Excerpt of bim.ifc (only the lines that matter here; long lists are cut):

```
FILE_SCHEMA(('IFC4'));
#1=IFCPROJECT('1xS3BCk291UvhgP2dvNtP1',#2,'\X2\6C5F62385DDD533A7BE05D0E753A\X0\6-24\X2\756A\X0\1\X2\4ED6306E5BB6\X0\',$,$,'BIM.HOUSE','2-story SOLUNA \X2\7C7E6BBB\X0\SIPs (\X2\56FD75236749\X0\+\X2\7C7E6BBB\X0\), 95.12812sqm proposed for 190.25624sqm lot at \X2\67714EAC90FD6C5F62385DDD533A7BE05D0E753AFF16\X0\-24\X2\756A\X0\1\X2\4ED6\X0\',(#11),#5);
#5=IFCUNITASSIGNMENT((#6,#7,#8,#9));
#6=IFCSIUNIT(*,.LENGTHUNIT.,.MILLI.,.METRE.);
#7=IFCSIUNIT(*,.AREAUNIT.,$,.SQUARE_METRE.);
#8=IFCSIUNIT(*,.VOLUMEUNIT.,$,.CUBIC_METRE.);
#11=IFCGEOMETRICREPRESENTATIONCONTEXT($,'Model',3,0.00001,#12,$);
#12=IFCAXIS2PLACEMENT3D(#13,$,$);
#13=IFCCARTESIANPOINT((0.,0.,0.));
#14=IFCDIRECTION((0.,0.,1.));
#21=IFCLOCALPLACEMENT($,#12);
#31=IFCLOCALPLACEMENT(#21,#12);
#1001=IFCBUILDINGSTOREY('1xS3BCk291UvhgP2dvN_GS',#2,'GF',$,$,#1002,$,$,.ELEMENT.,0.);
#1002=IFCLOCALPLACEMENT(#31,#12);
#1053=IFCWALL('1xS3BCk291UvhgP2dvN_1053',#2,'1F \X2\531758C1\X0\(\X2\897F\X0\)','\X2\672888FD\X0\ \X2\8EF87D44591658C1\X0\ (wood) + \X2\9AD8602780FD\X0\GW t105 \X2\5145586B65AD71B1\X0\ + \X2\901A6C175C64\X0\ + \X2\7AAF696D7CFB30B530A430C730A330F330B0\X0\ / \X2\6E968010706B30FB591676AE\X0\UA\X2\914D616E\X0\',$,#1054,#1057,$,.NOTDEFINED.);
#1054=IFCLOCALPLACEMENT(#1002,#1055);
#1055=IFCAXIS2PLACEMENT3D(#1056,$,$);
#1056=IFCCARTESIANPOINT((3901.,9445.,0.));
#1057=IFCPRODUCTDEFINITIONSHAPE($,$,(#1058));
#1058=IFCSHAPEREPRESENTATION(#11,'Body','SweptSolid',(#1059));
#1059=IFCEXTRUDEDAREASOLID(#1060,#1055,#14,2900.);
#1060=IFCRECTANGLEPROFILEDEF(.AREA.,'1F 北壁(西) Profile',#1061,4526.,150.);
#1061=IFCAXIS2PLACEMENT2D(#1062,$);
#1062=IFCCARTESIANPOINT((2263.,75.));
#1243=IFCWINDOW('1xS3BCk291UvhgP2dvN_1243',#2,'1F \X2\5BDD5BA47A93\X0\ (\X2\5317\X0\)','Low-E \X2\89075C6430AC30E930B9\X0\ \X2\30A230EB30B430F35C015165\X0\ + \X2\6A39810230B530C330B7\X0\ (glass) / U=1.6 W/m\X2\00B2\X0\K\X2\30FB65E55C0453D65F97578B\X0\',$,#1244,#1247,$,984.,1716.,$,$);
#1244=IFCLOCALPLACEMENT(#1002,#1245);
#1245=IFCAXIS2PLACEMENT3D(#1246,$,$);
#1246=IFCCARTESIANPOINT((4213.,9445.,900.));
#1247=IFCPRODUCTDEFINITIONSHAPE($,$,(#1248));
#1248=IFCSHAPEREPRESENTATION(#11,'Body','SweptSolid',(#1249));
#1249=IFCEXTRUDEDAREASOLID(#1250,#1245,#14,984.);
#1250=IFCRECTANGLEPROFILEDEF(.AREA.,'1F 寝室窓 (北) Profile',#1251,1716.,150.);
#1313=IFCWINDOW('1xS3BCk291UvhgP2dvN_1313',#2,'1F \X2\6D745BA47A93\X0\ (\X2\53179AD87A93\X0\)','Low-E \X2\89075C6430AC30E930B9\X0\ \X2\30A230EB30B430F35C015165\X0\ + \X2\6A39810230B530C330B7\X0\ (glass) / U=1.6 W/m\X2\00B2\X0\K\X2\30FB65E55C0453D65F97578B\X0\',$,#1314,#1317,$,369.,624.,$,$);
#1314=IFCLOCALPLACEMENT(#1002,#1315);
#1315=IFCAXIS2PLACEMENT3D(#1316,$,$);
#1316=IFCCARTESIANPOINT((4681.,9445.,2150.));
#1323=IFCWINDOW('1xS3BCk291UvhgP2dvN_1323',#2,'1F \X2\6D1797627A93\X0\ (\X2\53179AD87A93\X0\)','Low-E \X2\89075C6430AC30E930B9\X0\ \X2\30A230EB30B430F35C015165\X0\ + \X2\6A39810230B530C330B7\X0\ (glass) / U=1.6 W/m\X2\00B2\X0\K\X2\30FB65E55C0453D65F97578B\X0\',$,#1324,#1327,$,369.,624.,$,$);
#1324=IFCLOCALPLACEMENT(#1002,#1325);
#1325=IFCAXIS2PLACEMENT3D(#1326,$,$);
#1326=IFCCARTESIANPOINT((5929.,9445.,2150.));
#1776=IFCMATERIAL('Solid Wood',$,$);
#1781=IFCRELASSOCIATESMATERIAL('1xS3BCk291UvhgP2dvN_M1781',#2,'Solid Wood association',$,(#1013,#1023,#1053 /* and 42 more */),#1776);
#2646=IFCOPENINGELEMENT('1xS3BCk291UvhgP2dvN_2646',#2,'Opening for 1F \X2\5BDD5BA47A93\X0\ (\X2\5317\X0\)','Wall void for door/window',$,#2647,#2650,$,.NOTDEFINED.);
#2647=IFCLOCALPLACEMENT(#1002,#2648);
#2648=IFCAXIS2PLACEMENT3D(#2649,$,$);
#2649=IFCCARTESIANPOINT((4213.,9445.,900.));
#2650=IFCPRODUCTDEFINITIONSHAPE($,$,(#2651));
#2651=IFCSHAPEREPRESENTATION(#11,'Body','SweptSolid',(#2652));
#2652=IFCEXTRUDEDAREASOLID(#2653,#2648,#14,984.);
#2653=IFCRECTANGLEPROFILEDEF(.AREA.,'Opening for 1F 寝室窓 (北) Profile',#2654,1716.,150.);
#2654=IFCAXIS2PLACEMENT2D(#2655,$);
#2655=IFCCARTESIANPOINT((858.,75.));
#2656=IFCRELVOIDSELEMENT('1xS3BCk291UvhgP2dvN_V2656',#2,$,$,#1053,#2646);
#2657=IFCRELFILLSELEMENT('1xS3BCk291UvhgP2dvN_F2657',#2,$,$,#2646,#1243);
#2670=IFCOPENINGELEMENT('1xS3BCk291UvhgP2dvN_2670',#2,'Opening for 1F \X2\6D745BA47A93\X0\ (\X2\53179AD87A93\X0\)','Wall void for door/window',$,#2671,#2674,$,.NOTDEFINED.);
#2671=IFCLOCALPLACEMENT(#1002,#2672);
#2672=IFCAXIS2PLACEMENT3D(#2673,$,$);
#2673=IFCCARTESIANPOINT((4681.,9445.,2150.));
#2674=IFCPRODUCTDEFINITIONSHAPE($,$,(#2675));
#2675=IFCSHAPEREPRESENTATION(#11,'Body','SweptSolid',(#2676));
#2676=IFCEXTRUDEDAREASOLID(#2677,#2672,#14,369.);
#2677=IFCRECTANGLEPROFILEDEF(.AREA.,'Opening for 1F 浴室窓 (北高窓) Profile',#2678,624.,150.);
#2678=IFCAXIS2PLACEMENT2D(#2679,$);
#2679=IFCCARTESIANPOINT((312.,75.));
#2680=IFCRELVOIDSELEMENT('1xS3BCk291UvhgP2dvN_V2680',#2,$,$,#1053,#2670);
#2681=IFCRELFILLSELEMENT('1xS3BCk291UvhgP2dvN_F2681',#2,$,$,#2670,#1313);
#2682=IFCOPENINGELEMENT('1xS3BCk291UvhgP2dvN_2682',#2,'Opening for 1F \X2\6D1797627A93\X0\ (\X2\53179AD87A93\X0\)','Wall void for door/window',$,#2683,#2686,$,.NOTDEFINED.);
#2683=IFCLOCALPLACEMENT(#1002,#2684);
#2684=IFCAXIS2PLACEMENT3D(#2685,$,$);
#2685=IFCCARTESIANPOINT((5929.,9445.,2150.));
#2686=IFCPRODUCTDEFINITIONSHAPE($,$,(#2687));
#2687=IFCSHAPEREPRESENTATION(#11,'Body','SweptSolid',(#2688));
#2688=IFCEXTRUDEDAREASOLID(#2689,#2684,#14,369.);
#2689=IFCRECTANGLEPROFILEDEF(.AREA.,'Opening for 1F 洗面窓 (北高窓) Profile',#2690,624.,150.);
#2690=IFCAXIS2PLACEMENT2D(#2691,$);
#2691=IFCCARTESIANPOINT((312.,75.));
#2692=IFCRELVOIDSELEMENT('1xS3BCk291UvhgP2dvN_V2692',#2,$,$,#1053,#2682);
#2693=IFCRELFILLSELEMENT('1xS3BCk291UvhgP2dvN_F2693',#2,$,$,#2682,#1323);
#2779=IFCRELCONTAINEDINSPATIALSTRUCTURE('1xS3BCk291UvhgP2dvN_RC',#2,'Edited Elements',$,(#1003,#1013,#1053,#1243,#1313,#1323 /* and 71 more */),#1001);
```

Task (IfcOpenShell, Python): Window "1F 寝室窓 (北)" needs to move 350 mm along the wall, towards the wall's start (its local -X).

```python
import ifcopenshell
import ifcopenshell.api.geometry
import ifcopenshell.util.placement
import ifcopenshell.util.unit

model = ifcopenshell.open("bim.ifc")
unit_scale = ifcopenshell.util.unit.calculate_unit_scale(model)

window = model.by_guid("1xS3BCk291UvhgP2dvN_1243")
opening = window.FillsVoids[0].RelatingOpeningElement
wall = opening.VoidsElements[0].RelatingBuildingElement

wall_matrix = ifcopenshell.util.placement.get_local_placement(wall.ObjectPlacement)
shift = wall_matrix[:3, 0] * -0.35 / unit_scale
before = ifcopenshell.util.placement.get_local_placement(window.ObjectPlacement)[:3, 3].copy()

# The window is not placed relative to its opening, so move both.
for product in (opening, window):
    matrix = ifcopenshell.util.placement.get_local_placement(product.ObjectPlacement)
    matrix[:3, 3] += shift
    ifcopenshell.api.geometry.edit_object_placement(model, product=product, matrix=matrix, is_si=False)

after = ifcopenshell.util.placement.get_local_placement(window.ObjectPlacement)[:3, 3]
print("window moved by", (after - before).round(3) + 0.0)

model.write("bim_rev.ifc")
```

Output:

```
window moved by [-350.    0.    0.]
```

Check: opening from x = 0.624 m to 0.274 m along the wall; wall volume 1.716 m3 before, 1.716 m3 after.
